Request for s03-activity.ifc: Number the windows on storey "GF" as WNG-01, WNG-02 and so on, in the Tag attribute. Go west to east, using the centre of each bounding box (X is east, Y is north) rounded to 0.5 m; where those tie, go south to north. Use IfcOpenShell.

First a look at what the model holds.

```python
import ifcopenshell
import ifcopenshell.util.element
import ifcopenshell.util.placement

model = ifcopenshell.open("s03-activity.ifc")
print(model.schema)
storey = next(s for s in model.by_type("IfcBuildingStorey") if s.Name == "GF")
windows = [e for e in ifcopenshell.util.element.get_decomposition(storey) if e.is_a("IfcWindow")]
for e in sorted(windows, key=lambda e: e.id()):
    origin = ifcopenshell.util.placement.get_local_placement(e.ObjectPlacement)[:3, 3]
    print(e.id(), e.Tag, e.Name, origin.round(2) + 0.0, sep=" | ")
```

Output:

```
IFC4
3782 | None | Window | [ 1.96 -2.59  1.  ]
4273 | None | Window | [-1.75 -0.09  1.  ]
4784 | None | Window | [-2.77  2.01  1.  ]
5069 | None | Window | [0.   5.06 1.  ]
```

```python
import ifcopenshell
import ifcopenshell.geom
import ifcopenshell.util.element
import ifcopenshell.util.shape

model = ifcopenshell.open("s03-activity.ifc")
settings = ifcopenshell.geom.settings()
settings.set("use-world-coords", True)


def centre(element):
    shape = ifcopenshell.geom.create_shape(settings, element)
    return ifcopenshell.util.shape.get_bbox_centroid(shape.geometry)


storey = next(s for s in model.by_type("IfcBuildingStorey") if s.Name == "GF")
windows = [e for e in ifcopenshell.util.element.get_decomposition(storey) if e.is_a("IfcWindow")]

# Insertion points can sit at a corner or the storey origin, so sort by the geometry (in metres).
centres = {e: centre(e) for e in windows}
windows.sort(key=lambda e: (round(centres[e][0] / 0.5), centres[e][1]))

for i, e in enumerate(windows, start=1):
    number = f"WNG-{i:02d}"
    e.Tag = number
    print(e.id(), number)

model.write("s03-activity_edited.ifc")
```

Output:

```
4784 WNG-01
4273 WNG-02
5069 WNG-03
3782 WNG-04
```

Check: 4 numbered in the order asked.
